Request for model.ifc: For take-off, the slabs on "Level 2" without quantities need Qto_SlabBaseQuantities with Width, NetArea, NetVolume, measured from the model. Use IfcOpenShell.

First a look at what the model holds.

```python
import ifcopenshell
import ifcopenshell.util.element
import ifcopenshell.util.unit

model = ifcopenshell.open("model.ifc")
print(model.schema)
for unit_type in ("LENGTHUNIT", "AREAUNIT", "VOLUMEUNIT"):
    print(unit_type, ifcopenshell.util.unit.calculate_unit_scale(model, unit_type))
storey = next(s for s in model.by_type("IfcBuildingStorey") if s.Name == "Level 2")
slabs = [e for e in ifcopenshell.util.element.get_decomposition(storey) if e.is_a("IfcSlab")]
for e in sorted(slabs, key=lambda e: e.id()):
    print(e.id(), e.is_a(), e.Name, list(ifcopenshell.util.element.get_psets(e, qtos_only=True)), sep=" | ")
```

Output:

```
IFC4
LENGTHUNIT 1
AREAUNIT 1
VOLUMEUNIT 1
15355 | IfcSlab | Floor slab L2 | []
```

```python
import ifcopenshell
import ifcopenshell.api.pset
import ifcopenshell.geom
import ifcopenshell.util.element
import ifcopenshell.util.shape
import ifcopenshell.util.unit

model = ifcopenshell.open("model.ifc")
unit_scale = ifcopenshell.util.unit.calculate_unit_scale(model)
area_scale = ifcopenshell.util.unit.calculate_unit_scale(model, "AREAUNIT")
volume_scale = ifcopenshell.util.unit.calculate_unit_scale(model, "VOLUMEUNIT")
settings = ifcopenshell.geom.settings()

storey = next(s for s in model.by_type("IfcBuildingStorey") if s.Name == "Level 2")
slabs = [e for e in ifcopenshell.util.element.get_decomposition(storey) if e.is_a("IfcSlab")]

for e in sorted(slabs, key=lambda e: e.id()):
    if ifcopenshell.util.element.get_psets(e, qtos_only=True, should_inherit=False):
        continue
    # Geometry comes back in metres, in the element's own axes.
    shape = ifcopenshell.geom.create_shape(settings, e)
    values = {
        "Width": ifcopenshell.util.shape.get_z(shape.geometry) / unit_scale,
        "NetArea": ifcopenshell.util.shape.get_footprint_area(shape.geometry) / area_scale,
        "NetVolume": ifcopenshell.util.shape.get_volume(shape.geometry) / volume_scale,
    }
    qto = ifcopenshell.api.pset.add_qto(model, product=e, name="Qto_SlabBaseQuantities")
    ifcopenshell.api.pset.edit_qto(model, qto=qto, properties=values)
    print(e.id(), {k: round(v, 3) for k, v in values.items()})

model.write("model-out.ifc")
```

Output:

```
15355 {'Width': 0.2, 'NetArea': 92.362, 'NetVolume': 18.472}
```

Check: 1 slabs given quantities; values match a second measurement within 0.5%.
